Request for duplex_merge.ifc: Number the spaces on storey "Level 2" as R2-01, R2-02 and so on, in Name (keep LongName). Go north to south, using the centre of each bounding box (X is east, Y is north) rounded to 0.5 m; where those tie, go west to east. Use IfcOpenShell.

First a look at what the model holds.

```python
import ifcopenshell
import ifcopenshell.util.element
import ifcopenshell.util.placement

model = ifcopenshell.open("duplex_merge.ifc")
print(model.schema)
storey = next(s for s in model.by_type("IfcBuildingStorey") if s.Name == "Level 2")
spaces = [e for e in ifcopenshell.util.element.get_decomposition(storey) if e.is_a("IfcSpace")]
for e in sorted(spaces, key=lambda e: e.id()):
    origin = ifcopenshell.util.placement.get_local_placement(e.ObjectPlacement)[:3, 3]
    print(e.id(), e.Name, e.LongName, origin.round(2) + 0.0, sep=" | ")
```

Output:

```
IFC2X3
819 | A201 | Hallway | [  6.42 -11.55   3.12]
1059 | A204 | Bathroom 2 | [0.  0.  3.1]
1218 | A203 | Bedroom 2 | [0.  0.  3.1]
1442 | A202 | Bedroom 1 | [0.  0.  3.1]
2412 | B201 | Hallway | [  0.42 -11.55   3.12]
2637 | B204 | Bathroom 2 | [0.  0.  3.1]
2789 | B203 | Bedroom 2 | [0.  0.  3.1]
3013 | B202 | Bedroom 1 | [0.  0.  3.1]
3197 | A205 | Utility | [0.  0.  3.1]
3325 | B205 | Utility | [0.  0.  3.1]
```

```python
import ifcopenshell
import ifcopenshell.geom
import ifcopenshell.util.element
import ifcopenshell.util.shape

model = ifcopenshell.open("duplex_merge.ifc")
settings = ifcopenshell.geom.settings()
settings.set("use-world-coords", True)


def centre(element):
    shape = ifcopenshell.geom.create_shape(settings, element)
    return ifcopenshell.util.shape.get_bbox_centroid(shape.geometry)


storey = next(s for s in model.by_type("IfcBuildingStorey") if s.Name == "Level 2")
spaces = [e for e in ifcopenshell.util.element.get_decomposition(storey) if e.is_a("IfcSpace")]

# Insertion points can sit at a corner or the storey origin, so sort by the geometry (in metres).
centres = {e: centre(e) for e in spaces}
spaces.sort(key=lambda e: (-round(centres[e][1] / 0.5), centres[e][0]))

for i, e in enumerate(spaces, start=1):
    number = f"R2-{i:02d}"
    e.Name = number
    print(e.id(), number)

model.write("duplex_merge_rev.ifc")
```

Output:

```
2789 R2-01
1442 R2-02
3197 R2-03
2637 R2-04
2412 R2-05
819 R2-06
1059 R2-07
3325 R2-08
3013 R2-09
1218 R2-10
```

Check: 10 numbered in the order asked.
